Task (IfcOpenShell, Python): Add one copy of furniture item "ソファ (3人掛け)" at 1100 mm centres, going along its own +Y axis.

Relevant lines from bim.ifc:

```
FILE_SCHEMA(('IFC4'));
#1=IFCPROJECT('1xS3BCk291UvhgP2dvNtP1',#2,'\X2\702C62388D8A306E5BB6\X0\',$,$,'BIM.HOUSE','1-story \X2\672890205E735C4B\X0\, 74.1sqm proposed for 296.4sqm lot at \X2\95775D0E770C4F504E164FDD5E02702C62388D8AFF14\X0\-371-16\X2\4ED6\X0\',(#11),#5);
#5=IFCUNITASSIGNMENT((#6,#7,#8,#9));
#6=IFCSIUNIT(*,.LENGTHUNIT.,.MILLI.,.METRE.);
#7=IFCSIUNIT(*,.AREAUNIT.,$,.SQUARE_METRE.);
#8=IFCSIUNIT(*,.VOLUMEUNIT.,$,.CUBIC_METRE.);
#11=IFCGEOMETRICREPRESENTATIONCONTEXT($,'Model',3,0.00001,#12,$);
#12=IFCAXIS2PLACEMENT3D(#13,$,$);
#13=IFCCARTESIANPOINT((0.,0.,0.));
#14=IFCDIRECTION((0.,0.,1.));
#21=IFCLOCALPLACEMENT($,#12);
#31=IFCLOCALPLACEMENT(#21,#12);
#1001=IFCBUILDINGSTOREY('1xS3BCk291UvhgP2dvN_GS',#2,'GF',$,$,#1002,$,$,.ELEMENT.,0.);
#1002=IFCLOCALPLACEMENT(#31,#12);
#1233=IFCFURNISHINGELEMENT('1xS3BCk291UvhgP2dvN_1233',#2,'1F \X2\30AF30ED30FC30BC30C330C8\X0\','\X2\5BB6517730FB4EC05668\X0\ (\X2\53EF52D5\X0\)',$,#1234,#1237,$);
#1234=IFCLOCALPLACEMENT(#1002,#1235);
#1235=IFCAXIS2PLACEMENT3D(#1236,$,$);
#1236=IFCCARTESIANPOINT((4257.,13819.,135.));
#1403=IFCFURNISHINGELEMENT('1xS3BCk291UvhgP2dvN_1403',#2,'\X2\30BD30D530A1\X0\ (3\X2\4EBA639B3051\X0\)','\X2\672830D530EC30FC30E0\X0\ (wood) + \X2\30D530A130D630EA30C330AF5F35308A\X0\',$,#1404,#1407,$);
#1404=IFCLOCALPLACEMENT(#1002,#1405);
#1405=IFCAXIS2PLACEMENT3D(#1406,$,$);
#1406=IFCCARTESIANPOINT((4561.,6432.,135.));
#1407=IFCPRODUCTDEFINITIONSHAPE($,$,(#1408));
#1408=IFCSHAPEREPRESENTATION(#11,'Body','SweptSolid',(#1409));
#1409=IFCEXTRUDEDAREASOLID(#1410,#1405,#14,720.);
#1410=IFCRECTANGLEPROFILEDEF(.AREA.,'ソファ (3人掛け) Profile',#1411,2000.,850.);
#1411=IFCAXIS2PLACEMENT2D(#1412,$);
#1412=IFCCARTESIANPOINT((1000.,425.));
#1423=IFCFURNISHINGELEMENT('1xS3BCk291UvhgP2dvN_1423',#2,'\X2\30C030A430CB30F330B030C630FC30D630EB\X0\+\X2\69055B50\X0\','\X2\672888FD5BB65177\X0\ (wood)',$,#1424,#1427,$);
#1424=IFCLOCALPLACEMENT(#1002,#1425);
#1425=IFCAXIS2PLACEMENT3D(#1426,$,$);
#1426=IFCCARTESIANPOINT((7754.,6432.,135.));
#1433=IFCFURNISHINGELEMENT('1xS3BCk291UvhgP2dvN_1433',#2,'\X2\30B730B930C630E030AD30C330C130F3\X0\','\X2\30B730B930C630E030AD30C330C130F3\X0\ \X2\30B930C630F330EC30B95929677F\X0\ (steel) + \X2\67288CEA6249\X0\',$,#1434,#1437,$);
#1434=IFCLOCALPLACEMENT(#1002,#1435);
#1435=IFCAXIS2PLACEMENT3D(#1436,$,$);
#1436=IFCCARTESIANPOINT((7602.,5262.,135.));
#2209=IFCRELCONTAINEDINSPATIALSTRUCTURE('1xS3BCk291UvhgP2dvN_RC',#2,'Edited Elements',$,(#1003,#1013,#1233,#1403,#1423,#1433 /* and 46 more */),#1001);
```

```python
import ifcopenshell
import ifcopenshell.api.geometry
import ifcopenshell.api.root
import ifcopenshell.util.element
import ifcopenshell.util.placement

model = ifcopenshell.open("bim.ifc")


def reuse_history(source, copy):
    """copy_class also copies each property set's owner history, people and application; keep the originals."""
    for rel in copy.IsDefinedBy:
        if rel.is_a("IfcRelDefinesByProperties") and (history := rel.RelatingPropertyDefinition.OwnerHistory):
            rel.RelatingPropertyDefinition.OwnerHistory = source.OwnerHistory
            ifcopenshell.util.element.remove_deep2(model, history)


source = model.by_guid("1xS3BCk291UvhgP2dvN_1403")
base = ifcopenshell.util.placement.get_local_placement(source.ObjectPlacement)
step = base[:3, 1] * 1100.0

for i in range(1, 2):
    copy = ifcopenshell.api.root.copy_class(model, product=source)
    copy.Representation = ifcopenshell.util.element.copy_deep(
        model, source.Representation, exclude=["IfcGeometricRepresentationContext", "IfcRepresentationMap"]
    )
    reuse_history(source, copy)
    matrix = base.copy()
    matrix[:3, 3] += i * step
    print("added at", matrix[:3, 3].round(3) + 0.0)
    ifcopenshell.api.geometry.edit_object_placement(model, product=copy, matrix=matrix, is_si=False)

model.write("bim_edited.ifc")
```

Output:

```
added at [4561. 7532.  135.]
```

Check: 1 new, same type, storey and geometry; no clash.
